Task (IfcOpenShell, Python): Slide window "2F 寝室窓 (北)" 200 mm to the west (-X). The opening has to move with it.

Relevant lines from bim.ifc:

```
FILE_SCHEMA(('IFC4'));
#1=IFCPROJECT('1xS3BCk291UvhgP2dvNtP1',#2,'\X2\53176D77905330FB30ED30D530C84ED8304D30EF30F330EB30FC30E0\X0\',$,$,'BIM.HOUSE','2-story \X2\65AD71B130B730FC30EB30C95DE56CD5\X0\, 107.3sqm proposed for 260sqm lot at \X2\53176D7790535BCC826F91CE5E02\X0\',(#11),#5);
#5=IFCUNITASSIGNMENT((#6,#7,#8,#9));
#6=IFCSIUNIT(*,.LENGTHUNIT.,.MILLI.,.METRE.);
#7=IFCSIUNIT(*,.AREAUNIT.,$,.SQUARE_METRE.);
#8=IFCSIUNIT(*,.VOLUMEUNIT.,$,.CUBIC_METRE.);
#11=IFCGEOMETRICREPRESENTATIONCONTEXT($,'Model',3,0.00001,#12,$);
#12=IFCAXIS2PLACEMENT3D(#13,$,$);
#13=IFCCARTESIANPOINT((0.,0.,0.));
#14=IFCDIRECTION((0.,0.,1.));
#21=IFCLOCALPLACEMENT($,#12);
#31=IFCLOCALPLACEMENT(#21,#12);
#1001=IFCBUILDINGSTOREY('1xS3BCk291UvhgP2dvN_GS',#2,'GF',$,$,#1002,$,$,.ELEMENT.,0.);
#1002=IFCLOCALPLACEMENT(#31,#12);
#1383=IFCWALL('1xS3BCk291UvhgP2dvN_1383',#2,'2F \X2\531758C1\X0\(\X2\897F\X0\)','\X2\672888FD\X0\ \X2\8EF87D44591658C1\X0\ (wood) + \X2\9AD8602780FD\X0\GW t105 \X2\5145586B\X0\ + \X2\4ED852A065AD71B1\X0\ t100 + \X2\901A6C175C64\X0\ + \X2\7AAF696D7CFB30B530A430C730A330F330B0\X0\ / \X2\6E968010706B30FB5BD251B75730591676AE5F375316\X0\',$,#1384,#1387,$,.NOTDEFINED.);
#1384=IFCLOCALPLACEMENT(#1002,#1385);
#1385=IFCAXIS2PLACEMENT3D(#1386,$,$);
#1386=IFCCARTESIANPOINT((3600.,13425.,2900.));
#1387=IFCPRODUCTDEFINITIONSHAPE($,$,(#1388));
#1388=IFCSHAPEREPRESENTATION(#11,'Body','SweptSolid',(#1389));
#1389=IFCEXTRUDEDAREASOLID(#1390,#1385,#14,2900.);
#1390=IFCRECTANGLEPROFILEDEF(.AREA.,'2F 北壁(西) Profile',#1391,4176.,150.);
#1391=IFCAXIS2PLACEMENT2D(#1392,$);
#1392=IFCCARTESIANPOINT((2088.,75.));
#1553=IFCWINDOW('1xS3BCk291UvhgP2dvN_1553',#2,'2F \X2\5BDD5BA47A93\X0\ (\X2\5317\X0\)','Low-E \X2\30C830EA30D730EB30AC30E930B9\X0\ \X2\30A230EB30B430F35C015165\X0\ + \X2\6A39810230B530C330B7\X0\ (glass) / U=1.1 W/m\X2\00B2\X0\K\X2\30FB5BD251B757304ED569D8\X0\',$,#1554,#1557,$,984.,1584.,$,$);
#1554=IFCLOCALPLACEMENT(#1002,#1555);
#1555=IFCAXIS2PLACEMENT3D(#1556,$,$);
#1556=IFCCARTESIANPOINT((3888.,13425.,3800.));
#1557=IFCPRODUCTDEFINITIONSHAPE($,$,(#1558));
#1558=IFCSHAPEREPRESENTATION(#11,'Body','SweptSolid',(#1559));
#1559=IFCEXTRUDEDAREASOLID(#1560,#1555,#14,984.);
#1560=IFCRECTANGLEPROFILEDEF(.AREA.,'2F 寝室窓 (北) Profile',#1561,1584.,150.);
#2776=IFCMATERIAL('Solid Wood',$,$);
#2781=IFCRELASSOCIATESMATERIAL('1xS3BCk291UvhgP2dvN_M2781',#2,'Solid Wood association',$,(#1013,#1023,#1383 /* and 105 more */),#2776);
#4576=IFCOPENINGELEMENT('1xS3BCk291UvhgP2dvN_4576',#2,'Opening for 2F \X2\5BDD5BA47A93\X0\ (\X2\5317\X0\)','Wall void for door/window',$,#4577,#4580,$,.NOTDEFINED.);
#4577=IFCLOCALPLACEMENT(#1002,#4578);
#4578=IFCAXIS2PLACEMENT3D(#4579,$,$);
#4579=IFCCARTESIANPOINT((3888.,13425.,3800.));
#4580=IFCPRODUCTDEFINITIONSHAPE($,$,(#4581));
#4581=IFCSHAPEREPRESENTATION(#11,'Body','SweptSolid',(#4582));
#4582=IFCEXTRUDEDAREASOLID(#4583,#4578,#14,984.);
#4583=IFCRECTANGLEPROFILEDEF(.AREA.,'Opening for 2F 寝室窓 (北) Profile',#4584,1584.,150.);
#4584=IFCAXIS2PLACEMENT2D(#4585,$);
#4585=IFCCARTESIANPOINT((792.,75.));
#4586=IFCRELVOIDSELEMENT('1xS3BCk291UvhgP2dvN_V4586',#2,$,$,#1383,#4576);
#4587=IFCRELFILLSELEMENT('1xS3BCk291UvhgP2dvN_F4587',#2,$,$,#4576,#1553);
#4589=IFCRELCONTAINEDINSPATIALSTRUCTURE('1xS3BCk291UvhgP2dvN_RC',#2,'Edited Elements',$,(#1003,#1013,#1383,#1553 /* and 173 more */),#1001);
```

```python
import ifcopenshell
import ifcopenshell.api.geometry
import ifcopenshell.util.placement
import ifcopenshell.util.unit

model = ifcopenshell.open("bim.ifc")
unit_scale = ifcopenshell.util.unit.calculate_unit_scale(model)

window = model.by_guid("1xS3BCk291UvhgP2dvN_1553")
opening = window.FillsVoids[0].RelatingOpeningElement
wall = opening.VoidsElements[0].RelatingBuildingElement

wall_matrix = ifcopenshell.util.placement.get_local_placement(wall.ObjectPlacement)
shift = wall_matrix[:3, 0] * -0.2 / unit_scale
before = ifcopenshell.util.placement.get_local_placement(window.ObjectPlacement)[:3, 3].copy()

# The window is not placed relative to its opening, so move both.
for product in (opening, window):
    matrix = ifcopenshell.util.placement.get_local_placement(product.ObjectPlacement)
    matrix[:3, 3] += shift
    ifcopenshell.api.geometry.edit_object_placement(model, product=product, matrix=matrix, is_si=False)

after = ifcopenshell.util.placement.get_local_placement(window.ObjectPlacement)[:3, 3]
print("window moved by", (after - before).round(3) + 0.0)

model.write("bim_edited.ifc")
```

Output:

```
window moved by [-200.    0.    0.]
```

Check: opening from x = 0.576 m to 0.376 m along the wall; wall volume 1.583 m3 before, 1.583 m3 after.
